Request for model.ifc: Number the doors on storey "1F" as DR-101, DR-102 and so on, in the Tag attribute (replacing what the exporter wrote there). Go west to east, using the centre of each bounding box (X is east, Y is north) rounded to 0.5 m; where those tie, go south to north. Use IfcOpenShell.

First a look at what the model holds.

```python
import ifcopenshell
import ifcopenshell.util.element
import ifcopenshell.util.placement

model = ifcopenshell.open("model.ifc")
print(model.schema)
storey = next(s for s in model.by_type("IfcBuildingStorey") if s.Name == "1F")
doors = [e for e in ifcopenshell.util.element.get_decomposition(storey) if e.is_a("IfcDoor")]
for e in sorted(doors, key=lambda e: e.id()):
    origin = ifcopenshell.util.placement.get_local_placement(e.ObjectPlacement)[:3, 3]
    print(e.id(), e.Tag, e.Name, origin.round(2) + 0.0, sep=" | ")
```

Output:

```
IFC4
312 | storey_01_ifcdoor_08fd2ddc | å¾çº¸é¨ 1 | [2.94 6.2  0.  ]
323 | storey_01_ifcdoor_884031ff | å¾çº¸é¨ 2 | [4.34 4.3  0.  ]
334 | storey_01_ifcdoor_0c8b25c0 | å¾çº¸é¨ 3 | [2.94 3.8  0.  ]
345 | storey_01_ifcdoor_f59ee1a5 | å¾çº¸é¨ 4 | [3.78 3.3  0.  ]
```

```python
import ifcopenshell
import ifcopenshell.geom
import ifcopenshell.util.element
import ifcopenshell.util.shape

model = ifcopenshell.open("model.ifc")
settings = ifcopenshell.geom.settings()
settings.set("use-world-coords", True)


def centre(element):
    shape = ifcopenshell.geom.create_shape(settings, element)
    return ifcopenshell.util.shape.get_bbox_centroid(shape.geometry)


storey = next(s for s in model.by_type("IfcBuildingStorey") if s.Name == "1F")
doors = [e for e in ifcopenshell.util.element.get_decomposition(storey) if e.is_a("IfcDoor")]

# Insertion points can sit at a corner or the storey origin, so sort by the geometry (in metres).
centres = {e: centre(e) for e in doors}
doors.sort(key=lambda e: (round(centres[e][0] / 0.5), centres[e][1]))

for i, e in enumerate(doors, start=1):
    number = f"DR-1{i:02d}"
    e.Tag = number
    print(e.id(), number)

model.write("model_updated.ifc")
```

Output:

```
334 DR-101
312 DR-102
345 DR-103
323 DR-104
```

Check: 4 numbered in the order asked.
